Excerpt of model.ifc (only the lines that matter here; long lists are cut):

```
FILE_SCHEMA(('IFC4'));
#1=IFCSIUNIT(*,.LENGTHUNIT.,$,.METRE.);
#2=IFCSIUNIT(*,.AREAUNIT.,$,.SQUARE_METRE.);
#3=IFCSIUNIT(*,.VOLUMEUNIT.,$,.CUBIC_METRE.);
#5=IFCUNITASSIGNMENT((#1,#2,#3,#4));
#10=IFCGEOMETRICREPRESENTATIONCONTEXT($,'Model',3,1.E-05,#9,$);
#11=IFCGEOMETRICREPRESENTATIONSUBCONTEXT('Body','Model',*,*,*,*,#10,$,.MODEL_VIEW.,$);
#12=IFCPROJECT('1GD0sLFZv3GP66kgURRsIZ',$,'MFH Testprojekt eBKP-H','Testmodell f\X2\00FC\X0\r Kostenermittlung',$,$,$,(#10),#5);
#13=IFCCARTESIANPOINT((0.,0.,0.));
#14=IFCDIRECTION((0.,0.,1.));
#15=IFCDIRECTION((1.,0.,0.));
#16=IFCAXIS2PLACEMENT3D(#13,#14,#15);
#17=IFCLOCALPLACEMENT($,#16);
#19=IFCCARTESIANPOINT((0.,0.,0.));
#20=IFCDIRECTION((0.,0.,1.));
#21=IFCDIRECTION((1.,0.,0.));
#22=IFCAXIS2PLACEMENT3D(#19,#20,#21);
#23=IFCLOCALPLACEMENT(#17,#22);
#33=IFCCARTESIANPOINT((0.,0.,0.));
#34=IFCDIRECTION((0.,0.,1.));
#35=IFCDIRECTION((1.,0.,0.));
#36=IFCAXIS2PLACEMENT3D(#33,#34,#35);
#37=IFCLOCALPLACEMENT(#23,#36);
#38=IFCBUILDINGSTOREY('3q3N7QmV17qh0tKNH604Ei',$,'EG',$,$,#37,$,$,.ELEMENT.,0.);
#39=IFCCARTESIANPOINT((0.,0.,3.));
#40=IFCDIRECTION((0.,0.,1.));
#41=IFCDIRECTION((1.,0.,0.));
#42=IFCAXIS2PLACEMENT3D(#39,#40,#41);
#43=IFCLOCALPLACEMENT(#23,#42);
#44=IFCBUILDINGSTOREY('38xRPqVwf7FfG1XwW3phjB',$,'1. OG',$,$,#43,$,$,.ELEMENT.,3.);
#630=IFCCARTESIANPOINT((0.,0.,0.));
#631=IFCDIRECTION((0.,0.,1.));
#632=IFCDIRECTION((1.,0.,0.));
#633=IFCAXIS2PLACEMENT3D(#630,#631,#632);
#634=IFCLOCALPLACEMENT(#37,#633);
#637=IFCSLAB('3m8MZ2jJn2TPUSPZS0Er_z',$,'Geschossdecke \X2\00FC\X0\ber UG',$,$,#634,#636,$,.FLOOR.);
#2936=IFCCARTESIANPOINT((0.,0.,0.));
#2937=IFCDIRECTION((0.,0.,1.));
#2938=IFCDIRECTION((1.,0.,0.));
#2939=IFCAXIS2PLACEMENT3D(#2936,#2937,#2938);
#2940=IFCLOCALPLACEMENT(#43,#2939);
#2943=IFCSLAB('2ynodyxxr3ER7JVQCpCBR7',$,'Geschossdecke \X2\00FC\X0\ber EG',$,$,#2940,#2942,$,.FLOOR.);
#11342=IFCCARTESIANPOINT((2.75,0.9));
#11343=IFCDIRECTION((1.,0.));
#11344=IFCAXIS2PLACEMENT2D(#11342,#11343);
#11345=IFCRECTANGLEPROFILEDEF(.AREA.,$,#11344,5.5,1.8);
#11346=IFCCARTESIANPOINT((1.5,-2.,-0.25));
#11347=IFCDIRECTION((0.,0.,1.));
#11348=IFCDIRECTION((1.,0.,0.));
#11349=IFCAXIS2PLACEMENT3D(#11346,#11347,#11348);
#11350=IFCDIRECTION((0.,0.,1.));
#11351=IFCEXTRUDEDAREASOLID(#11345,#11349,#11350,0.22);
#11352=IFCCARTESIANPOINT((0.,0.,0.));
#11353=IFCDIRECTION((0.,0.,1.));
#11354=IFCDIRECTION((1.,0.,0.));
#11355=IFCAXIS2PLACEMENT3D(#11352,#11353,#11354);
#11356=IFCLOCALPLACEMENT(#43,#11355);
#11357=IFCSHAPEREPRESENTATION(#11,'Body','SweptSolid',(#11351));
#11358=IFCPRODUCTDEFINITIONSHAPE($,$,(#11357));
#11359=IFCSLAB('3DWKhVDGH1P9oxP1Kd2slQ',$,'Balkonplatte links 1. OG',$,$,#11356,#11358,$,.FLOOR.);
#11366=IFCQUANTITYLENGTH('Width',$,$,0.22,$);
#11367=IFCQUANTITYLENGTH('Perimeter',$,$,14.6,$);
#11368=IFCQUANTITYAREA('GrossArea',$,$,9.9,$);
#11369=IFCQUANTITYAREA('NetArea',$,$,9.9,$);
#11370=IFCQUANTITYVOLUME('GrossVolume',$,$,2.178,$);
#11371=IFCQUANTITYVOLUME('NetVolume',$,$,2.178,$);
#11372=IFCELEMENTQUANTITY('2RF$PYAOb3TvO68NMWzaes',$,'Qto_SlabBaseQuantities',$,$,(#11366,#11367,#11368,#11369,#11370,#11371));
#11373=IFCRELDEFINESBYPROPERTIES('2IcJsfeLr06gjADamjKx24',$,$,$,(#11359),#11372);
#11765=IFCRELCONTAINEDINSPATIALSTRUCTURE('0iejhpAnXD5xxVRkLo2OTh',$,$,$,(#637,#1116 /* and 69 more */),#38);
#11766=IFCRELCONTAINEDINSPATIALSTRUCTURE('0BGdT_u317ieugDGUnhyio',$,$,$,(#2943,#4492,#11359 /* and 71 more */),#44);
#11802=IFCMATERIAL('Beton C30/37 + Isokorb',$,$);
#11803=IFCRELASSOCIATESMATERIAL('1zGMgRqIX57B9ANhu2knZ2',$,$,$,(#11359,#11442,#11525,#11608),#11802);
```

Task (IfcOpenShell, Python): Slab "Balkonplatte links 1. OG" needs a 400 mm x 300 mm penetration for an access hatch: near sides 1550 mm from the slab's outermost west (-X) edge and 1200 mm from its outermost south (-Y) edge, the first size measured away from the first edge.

```python
import numpy as np
import ifcopenshell
import ifcopenshell.api.feature
import ifcopenshell.api.geometry
import ifcopenshell.api.pset
import ifcopenshell.api.root
import ifcopenshell.geom
import ifcopenshell.util.element
import ifcopenshell.util.placement
import ifcopenshell.util.representation
import ifcopenshell.util.shape
import ifcopenshell.util.unit

model = ifcopenshell.open("model.ifc")
unit_scale = ifcopenshell.util.unit.calculate_unit_scale(model)
area_scale = ifcopenshell.util.unit.calculate_unit_scale(model, "AREAUNIT")
volume_scale = ifcopenshell.util.unit.calculate_unit_scale(model, "VOLUMEUNIT")
settings = ifcopenshell.geom.settings()


def volume(element):
    """Net volume in cubic metres, openings subtracted."""
    shape = ifcopenshell.geom.create_shape(settings, element)
    return ifcopenshell.util.shape.get_volume(shape.geometry)


slab = model.by_guid("3DWKhVDGH1P9oxP1Kd2slQ")
before = volume(slab)

# Extent in the slab's own axes, in metres. The edges named are its -X and -Y sides.
slab_shape = ifcopenshell.geom.create_shape(settings, slab)
vertices = ifcopenshell.util.shape.get_vertices(slab_shape.geometry)
x_min, y_min, bottom = vertices.min(axis=0)
top = vertices[:, 2].max()

opening = ifcopenshell.api.root.create_entity(model, ifc_class="IfcOpeningElement", name="Access hatch opening", predefined_type="OPENING")
context = ifcopenshell.util.representation.get_context(model, "Model", "Body", "MODEL_VIEW")
width, depth = 0.4, 0.3
outline = [(0.0, 0.0), (width, 0.0), (width, depth), (0.0, depth), (0.0, 0.0)]
# Overshoot both faces by 50 mm so the cut is clean.
shape = ifcopenshell.api.geometry.add_slab_representation(
    model, context=context, depth=top - bottom + 0.1, polyline=outline
)
ifcopenshell.api.geometry.assign_representation(model, product=opening, representation=shape)

matrix = ifcopenshell.util.placement.get_local_placement(slab.ObjectPlacement)
matrix[:, 3] = matrix @ np.append(np.array([x_min + 1.55, y_min + 1.2, bottom - 0.05]) / unit_scale, 1.0)
ifcopenshell.api.geometry.edit_object_placement(model, product=opening, matrix=matrix, is_si=False)
ifcopenshell.api.feature.add_feature(model, feature=opening, element=slab)

after = volume(slab)

# Update the slab's stored quantities.
qto = model.by_id(ifcopenshell.util.element.get_pset(slab, "Qto_SlabBaseQuantities", should_inherit=False)["id"])
ifcopenshell.api.pset.edit_qto(model, qto=qto, properties={
    "NetArea": after / (top - bottom) / area_scale,
    "NetVolume": after / volume_scale,
})

print(f"slab volume {before:.3f} -> {after:.3f} m3")

model.write("model_updated.ifc")
```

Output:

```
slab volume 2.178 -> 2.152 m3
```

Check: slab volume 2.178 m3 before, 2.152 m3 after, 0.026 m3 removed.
